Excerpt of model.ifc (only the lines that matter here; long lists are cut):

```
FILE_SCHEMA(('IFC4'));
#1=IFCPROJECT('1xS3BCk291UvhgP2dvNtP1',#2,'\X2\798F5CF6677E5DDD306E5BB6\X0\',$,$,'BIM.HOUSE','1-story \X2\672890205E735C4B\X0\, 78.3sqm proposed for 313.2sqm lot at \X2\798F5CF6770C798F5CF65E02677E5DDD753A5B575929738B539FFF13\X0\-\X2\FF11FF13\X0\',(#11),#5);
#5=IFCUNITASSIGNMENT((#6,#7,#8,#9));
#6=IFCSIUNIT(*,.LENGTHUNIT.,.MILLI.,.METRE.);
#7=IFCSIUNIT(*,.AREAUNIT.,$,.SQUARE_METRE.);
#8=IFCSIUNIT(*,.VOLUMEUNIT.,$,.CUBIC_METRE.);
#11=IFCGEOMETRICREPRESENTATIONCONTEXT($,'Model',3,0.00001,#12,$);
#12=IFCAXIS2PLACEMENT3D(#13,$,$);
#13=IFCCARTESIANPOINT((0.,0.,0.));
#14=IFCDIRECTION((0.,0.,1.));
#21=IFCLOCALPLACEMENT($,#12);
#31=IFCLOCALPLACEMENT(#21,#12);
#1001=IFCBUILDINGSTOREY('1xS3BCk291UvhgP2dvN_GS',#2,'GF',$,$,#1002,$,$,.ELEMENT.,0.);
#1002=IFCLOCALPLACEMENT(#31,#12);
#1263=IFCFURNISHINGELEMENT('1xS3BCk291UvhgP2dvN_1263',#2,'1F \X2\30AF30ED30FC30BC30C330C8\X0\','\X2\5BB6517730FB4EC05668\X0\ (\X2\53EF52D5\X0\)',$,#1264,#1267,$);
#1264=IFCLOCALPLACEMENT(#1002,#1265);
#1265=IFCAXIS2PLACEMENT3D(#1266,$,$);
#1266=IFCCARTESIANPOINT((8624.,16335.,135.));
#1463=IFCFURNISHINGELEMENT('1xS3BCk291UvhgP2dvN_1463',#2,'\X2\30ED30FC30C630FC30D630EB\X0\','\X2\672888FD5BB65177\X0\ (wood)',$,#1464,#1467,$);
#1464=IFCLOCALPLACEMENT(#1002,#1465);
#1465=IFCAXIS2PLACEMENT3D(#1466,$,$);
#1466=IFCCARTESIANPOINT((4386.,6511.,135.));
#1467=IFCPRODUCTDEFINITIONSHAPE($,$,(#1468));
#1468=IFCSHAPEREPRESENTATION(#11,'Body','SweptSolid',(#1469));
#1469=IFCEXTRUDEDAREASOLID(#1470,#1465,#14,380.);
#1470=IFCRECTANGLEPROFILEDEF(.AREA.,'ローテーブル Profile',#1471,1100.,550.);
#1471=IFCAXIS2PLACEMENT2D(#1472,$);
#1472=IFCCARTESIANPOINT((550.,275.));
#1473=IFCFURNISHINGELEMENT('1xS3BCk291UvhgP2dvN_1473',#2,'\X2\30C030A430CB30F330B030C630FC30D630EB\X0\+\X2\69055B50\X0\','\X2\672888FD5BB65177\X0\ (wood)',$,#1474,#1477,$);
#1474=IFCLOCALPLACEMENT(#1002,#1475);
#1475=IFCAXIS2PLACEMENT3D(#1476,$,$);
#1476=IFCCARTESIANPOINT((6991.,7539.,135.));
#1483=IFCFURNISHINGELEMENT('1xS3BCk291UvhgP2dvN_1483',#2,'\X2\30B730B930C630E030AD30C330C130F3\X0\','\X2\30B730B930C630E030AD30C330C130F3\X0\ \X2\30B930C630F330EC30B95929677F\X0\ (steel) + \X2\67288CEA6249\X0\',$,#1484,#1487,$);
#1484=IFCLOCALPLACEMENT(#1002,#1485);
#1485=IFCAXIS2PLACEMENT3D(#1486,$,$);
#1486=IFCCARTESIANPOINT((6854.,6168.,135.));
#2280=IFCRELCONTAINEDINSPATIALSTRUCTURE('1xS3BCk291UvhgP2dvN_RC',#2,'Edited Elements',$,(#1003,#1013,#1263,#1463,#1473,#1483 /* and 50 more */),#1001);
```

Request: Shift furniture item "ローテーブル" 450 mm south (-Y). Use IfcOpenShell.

```python
import ifcopenshell
import ifcopenshell.api.geometry
import ifcopenshell.util.placement
import ifcopenshell.util.unit

model = ifcopenshell.open("model.ifc")
unit_scale = ifcopenshell.util.unit.calculate_unit_scale(model)

item = model.by_guid("1xS3BCk291UvhgP2dvN_1463")
matrix = ifcopenshell.util.placement.get_local_placement(item.ObjectPlacement)
matrix[1, 3] -= 0.45 / unit_scale
ifcopenshell.api.geometry.edit_object_placement(model, product=item, matrix=matrix, is_si=False)

print(ifcopenshell.util.placement.get_local_placement(item.ObjectPlacement).round(3) + 0.0)

model.write("model_rev.ifc")
```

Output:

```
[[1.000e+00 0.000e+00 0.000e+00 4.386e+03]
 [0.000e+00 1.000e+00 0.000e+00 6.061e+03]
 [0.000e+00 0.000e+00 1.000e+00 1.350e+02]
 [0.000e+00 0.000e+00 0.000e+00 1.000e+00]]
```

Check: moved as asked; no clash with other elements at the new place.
